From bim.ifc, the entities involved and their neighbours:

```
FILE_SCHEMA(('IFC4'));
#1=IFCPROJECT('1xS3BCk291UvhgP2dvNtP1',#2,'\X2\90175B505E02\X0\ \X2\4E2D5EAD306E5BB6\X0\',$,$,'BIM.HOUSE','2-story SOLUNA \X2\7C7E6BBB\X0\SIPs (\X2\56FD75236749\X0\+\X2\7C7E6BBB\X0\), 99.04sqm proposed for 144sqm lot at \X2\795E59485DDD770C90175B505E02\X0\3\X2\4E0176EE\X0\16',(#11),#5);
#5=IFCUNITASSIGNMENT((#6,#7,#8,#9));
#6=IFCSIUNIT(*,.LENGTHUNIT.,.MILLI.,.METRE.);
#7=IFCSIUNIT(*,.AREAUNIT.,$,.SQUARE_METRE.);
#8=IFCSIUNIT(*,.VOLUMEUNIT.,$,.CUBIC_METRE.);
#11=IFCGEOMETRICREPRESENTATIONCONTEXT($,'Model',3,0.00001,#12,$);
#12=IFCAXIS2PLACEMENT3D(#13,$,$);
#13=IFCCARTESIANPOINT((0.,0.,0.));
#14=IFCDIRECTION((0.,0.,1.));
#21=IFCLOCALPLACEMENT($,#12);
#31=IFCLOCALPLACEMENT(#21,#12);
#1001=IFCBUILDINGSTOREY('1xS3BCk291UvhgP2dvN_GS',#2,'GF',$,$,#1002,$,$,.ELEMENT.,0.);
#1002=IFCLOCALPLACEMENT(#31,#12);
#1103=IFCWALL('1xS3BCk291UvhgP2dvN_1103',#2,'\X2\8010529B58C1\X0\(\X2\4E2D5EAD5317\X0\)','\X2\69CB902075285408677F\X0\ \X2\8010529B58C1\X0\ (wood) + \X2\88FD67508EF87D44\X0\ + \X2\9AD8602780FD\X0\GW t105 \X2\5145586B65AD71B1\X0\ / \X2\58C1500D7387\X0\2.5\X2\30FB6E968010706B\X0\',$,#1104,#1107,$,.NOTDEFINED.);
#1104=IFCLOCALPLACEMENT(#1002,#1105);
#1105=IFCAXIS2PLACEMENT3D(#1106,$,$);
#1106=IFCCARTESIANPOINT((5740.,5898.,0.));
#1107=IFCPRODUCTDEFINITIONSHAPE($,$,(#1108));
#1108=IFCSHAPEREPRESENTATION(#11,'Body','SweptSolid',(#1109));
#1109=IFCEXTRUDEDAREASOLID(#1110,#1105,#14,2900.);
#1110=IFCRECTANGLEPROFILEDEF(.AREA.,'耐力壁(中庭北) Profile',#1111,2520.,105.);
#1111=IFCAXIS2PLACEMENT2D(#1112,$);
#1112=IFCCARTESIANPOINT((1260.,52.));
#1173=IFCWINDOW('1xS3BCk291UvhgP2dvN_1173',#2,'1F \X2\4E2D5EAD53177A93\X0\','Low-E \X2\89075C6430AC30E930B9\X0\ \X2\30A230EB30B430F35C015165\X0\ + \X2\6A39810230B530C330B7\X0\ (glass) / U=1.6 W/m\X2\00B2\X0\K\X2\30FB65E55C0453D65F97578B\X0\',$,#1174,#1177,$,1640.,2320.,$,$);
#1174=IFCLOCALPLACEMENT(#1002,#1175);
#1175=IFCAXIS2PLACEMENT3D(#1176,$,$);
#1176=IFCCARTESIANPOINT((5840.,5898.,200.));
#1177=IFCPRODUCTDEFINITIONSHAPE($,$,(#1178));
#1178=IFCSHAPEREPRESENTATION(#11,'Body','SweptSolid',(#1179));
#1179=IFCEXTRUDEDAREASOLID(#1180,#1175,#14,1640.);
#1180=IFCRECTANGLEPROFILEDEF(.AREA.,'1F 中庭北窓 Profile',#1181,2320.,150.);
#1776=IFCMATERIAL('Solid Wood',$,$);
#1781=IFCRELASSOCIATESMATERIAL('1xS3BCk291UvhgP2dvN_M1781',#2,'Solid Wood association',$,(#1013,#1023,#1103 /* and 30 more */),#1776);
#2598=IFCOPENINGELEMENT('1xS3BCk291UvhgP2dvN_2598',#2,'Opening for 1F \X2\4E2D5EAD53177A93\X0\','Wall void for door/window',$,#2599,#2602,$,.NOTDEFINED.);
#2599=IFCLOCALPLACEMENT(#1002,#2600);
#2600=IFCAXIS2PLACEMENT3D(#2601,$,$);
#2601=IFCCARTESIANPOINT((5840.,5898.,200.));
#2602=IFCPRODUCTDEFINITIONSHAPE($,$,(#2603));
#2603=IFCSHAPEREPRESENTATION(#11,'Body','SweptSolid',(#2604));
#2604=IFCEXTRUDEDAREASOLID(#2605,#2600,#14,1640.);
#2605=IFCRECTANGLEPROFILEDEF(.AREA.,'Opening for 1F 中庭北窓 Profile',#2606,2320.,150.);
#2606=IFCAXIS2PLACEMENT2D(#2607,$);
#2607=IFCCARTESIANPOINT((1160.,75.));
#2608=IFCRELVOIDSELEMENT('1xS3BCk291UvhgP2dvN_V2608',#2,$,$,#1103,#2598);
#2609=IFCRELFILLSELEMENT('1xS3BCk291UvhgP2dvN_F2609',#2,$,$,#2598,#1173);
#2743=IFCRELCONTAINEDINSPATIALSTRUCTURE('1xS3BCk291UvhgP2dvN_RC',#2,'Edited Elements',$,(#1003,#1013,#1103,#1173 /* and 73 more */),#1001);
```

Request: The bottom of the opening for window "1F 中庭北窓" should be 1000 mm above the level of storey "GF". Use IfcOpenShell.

```python
import numpy as np
import ifcopenshell
import ifcopenshell.api.geometry
import ifcopenshell.geom
import ifcopenshell.util.element
import ifcopenshell.util.placement
import ifcopenshell.util.shape
import ifcopenshell.util.unit

model = ifcopenshell.open("bim.ifc")
unit_scale = ifcopenshell.util.unit.calculate_unit_scale(model)

window = model.by_guid("1xS3BCk291UvhgP2dvN_1173")
opening = window.FillsVoids[0].RelatingOpeningElement
storey = ifcopenshell.util.element.get_container(window, ifc_class="IfcBuildingStorey")
level = ifcopenshell.util.placement.get_local_placement(storey.ObjectPlacement)[2, 3]

# The opening's origin need not be at the sill, so measure its lowest point.
shape = ifcopenshell.geom.create_shape(ifcopenshell.geom.settings(), opening)
bottom = ifcopenshell.util.shape.get_shape_bottom_elevation(shape, shape.geometry) / unit_scale
dz = level + 1000.0 - bottom

shift = np.array([0.0, 0.0, dz])
# The window is not placed relative to its opening, so move both.
for product in (opening, window):
    matrix = ifcopenshell.util.placement.get_local_placement(product.ObjectPlacement)
    matrix[:3, 3] += shift
    ifcopenshell.api.geometry.edit_object_placement(model, product=product, matrix=matrix, is_si=False)

print(f"moved by {dz * unit_scale:+.3f} m")

model.write("bim_rev.ifc")
```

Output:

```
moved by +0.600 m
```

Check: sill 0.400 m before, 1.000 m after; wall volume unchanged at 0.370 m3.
